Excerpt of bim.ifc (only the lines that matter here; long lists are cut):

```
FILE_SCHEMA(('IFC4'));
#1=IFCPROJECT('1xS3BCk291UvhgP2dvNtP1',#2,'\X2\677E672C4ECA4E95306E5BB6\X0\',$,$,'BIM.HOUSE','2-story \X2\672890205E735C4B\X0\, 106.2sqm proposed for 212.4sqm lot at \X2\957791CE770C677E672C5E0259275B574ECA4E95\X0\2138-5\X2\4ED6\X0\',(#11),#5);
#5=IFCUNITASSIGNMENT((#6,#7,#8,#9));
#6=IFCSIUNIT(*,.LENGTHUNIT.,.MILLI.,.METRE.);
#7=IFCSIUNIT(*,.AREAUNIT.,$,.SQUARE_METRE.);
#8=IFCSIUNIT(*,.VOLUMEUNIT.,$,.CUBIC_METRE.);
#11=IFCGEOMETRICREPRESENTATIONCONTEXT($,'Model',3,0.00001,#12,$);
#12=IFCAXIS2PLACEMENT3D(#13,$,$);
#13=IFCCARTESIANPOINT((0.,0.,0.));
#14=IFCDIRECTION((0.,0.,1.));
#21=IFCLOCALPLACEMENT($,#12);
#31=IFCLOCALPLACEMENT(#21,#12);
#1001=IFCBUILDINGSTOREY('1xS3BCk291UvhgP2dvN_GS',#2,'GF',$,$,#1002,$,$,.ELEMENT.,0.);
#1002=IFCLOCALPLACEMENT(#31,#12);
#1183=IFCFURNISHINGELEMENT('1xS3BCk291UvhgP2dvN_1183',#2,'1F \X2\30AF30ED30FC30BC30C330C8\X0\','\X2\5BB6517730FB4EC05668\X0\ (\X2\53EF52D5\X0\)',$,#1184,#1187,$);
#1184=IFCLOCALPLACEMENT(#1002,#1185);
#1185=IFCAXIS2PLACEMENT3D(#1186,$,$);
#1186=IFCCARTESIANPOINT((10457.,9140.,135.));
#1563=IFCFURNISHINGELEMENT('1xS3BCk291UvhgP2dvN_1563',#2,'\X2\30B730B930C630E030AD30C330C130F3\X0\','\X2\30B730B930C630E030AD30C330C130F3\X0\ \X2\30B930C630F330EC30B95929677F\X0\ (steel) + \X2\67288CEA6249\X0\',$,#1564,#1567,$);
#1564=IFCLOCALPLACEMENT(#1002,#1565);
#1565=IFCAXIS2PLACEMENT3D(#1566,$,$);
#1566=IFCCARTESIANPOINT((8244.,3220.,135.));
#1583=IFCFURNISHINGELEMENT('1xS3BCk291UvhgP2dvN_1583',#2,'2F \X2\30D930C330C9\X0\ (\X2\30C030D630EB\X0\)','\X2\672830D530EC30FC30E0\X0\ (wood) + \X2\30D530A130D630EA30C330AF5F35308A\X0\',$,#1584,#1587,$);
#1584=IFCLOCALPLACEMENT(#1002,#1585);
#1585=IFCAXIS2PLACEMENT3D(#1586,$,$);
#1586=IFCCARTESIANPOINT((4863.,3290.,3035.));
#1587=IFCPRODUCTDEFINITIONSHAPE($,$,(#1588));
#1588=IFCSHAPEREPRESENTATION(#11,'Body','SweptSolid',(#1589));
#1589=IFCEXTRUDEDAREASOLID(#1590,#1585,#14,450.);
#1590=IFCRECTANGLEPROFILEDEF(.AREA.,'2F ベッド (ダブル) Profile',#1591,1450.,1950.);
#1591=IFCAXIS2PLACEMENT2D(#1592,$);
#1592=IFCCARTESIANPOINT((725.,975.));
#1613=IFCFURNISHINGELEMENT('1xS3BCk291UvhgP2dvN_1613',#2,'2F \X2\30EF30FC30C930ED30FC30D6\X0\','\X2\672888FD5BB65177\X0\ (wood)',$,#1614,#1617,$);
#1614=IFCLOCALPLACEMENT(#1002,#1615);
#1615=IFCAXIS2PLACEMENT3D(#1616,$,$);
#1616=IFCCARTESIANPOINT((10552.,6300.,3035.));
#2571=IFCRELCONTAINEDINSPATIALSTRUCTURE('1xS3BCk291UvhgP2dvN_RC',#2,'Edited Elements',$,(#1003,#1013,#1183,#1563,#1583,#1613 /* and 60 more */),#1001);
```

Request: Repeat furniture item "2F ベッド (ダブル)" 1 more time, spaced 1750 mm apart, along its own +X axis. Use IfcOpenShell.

```python
import ifcopenshell
import ifcopenshell.api.geometry
import ifcopenshell.api.root
import ifcopenshell.util.element
import ifcopenshell.util.placement
import ifcopenshell.util.unit

model = ifcopenshell.open("bim.ifc")
unit_scale = ifcopenshell.util.unit.calculate_unit_scale(model)


def reuse_history(source, copy):
    """copy_class also copies each property set's owner history, people and application; keep the originals."""
    for rel in copy.IsDefinedBy:
        if rel.is_a("IfcRelDefinesByProperties") and (history := rel.RelatingPropertyDefinition.OwnerHistory):
            rel.RelatingPropertyDefinition.OwnerHistory = source.OwnerHistory
            ifcopenshell.util.element.remove_deep2(model, history)


source = model.by_guid("1xS3BCk291UvhgP2dvN_1583")
base = ifcopenshell.util.placement.get_local_placement(source.ObjectPlacement)
step = base[:3, 0] * 1.75 / unit_scale

for i in range(1, 2):
    copy = ifcopenshell.api.root.copy_class(model, product=source)
    copy.Representation = ifcopenshell.util.element.copy_deep(
        model, source.Representation, exclude=["IfcGeometricRepresentationContext", "IfcRepresentationMap"]
    )
    reuse_history(source, copy)
    matrix = base.copy()
    matrix[:3, 3] += i * step
    print("added at", matrix[:3, 3].round(3) + 0.0)
    ifcopenshell.api.geometry.edit_object_placement(model, product=copy, matrix=matrix, is_si=False)

model.write("bim_rev.ifc")
```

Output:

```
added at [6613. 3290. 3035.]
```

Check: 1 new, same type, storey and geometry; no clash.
